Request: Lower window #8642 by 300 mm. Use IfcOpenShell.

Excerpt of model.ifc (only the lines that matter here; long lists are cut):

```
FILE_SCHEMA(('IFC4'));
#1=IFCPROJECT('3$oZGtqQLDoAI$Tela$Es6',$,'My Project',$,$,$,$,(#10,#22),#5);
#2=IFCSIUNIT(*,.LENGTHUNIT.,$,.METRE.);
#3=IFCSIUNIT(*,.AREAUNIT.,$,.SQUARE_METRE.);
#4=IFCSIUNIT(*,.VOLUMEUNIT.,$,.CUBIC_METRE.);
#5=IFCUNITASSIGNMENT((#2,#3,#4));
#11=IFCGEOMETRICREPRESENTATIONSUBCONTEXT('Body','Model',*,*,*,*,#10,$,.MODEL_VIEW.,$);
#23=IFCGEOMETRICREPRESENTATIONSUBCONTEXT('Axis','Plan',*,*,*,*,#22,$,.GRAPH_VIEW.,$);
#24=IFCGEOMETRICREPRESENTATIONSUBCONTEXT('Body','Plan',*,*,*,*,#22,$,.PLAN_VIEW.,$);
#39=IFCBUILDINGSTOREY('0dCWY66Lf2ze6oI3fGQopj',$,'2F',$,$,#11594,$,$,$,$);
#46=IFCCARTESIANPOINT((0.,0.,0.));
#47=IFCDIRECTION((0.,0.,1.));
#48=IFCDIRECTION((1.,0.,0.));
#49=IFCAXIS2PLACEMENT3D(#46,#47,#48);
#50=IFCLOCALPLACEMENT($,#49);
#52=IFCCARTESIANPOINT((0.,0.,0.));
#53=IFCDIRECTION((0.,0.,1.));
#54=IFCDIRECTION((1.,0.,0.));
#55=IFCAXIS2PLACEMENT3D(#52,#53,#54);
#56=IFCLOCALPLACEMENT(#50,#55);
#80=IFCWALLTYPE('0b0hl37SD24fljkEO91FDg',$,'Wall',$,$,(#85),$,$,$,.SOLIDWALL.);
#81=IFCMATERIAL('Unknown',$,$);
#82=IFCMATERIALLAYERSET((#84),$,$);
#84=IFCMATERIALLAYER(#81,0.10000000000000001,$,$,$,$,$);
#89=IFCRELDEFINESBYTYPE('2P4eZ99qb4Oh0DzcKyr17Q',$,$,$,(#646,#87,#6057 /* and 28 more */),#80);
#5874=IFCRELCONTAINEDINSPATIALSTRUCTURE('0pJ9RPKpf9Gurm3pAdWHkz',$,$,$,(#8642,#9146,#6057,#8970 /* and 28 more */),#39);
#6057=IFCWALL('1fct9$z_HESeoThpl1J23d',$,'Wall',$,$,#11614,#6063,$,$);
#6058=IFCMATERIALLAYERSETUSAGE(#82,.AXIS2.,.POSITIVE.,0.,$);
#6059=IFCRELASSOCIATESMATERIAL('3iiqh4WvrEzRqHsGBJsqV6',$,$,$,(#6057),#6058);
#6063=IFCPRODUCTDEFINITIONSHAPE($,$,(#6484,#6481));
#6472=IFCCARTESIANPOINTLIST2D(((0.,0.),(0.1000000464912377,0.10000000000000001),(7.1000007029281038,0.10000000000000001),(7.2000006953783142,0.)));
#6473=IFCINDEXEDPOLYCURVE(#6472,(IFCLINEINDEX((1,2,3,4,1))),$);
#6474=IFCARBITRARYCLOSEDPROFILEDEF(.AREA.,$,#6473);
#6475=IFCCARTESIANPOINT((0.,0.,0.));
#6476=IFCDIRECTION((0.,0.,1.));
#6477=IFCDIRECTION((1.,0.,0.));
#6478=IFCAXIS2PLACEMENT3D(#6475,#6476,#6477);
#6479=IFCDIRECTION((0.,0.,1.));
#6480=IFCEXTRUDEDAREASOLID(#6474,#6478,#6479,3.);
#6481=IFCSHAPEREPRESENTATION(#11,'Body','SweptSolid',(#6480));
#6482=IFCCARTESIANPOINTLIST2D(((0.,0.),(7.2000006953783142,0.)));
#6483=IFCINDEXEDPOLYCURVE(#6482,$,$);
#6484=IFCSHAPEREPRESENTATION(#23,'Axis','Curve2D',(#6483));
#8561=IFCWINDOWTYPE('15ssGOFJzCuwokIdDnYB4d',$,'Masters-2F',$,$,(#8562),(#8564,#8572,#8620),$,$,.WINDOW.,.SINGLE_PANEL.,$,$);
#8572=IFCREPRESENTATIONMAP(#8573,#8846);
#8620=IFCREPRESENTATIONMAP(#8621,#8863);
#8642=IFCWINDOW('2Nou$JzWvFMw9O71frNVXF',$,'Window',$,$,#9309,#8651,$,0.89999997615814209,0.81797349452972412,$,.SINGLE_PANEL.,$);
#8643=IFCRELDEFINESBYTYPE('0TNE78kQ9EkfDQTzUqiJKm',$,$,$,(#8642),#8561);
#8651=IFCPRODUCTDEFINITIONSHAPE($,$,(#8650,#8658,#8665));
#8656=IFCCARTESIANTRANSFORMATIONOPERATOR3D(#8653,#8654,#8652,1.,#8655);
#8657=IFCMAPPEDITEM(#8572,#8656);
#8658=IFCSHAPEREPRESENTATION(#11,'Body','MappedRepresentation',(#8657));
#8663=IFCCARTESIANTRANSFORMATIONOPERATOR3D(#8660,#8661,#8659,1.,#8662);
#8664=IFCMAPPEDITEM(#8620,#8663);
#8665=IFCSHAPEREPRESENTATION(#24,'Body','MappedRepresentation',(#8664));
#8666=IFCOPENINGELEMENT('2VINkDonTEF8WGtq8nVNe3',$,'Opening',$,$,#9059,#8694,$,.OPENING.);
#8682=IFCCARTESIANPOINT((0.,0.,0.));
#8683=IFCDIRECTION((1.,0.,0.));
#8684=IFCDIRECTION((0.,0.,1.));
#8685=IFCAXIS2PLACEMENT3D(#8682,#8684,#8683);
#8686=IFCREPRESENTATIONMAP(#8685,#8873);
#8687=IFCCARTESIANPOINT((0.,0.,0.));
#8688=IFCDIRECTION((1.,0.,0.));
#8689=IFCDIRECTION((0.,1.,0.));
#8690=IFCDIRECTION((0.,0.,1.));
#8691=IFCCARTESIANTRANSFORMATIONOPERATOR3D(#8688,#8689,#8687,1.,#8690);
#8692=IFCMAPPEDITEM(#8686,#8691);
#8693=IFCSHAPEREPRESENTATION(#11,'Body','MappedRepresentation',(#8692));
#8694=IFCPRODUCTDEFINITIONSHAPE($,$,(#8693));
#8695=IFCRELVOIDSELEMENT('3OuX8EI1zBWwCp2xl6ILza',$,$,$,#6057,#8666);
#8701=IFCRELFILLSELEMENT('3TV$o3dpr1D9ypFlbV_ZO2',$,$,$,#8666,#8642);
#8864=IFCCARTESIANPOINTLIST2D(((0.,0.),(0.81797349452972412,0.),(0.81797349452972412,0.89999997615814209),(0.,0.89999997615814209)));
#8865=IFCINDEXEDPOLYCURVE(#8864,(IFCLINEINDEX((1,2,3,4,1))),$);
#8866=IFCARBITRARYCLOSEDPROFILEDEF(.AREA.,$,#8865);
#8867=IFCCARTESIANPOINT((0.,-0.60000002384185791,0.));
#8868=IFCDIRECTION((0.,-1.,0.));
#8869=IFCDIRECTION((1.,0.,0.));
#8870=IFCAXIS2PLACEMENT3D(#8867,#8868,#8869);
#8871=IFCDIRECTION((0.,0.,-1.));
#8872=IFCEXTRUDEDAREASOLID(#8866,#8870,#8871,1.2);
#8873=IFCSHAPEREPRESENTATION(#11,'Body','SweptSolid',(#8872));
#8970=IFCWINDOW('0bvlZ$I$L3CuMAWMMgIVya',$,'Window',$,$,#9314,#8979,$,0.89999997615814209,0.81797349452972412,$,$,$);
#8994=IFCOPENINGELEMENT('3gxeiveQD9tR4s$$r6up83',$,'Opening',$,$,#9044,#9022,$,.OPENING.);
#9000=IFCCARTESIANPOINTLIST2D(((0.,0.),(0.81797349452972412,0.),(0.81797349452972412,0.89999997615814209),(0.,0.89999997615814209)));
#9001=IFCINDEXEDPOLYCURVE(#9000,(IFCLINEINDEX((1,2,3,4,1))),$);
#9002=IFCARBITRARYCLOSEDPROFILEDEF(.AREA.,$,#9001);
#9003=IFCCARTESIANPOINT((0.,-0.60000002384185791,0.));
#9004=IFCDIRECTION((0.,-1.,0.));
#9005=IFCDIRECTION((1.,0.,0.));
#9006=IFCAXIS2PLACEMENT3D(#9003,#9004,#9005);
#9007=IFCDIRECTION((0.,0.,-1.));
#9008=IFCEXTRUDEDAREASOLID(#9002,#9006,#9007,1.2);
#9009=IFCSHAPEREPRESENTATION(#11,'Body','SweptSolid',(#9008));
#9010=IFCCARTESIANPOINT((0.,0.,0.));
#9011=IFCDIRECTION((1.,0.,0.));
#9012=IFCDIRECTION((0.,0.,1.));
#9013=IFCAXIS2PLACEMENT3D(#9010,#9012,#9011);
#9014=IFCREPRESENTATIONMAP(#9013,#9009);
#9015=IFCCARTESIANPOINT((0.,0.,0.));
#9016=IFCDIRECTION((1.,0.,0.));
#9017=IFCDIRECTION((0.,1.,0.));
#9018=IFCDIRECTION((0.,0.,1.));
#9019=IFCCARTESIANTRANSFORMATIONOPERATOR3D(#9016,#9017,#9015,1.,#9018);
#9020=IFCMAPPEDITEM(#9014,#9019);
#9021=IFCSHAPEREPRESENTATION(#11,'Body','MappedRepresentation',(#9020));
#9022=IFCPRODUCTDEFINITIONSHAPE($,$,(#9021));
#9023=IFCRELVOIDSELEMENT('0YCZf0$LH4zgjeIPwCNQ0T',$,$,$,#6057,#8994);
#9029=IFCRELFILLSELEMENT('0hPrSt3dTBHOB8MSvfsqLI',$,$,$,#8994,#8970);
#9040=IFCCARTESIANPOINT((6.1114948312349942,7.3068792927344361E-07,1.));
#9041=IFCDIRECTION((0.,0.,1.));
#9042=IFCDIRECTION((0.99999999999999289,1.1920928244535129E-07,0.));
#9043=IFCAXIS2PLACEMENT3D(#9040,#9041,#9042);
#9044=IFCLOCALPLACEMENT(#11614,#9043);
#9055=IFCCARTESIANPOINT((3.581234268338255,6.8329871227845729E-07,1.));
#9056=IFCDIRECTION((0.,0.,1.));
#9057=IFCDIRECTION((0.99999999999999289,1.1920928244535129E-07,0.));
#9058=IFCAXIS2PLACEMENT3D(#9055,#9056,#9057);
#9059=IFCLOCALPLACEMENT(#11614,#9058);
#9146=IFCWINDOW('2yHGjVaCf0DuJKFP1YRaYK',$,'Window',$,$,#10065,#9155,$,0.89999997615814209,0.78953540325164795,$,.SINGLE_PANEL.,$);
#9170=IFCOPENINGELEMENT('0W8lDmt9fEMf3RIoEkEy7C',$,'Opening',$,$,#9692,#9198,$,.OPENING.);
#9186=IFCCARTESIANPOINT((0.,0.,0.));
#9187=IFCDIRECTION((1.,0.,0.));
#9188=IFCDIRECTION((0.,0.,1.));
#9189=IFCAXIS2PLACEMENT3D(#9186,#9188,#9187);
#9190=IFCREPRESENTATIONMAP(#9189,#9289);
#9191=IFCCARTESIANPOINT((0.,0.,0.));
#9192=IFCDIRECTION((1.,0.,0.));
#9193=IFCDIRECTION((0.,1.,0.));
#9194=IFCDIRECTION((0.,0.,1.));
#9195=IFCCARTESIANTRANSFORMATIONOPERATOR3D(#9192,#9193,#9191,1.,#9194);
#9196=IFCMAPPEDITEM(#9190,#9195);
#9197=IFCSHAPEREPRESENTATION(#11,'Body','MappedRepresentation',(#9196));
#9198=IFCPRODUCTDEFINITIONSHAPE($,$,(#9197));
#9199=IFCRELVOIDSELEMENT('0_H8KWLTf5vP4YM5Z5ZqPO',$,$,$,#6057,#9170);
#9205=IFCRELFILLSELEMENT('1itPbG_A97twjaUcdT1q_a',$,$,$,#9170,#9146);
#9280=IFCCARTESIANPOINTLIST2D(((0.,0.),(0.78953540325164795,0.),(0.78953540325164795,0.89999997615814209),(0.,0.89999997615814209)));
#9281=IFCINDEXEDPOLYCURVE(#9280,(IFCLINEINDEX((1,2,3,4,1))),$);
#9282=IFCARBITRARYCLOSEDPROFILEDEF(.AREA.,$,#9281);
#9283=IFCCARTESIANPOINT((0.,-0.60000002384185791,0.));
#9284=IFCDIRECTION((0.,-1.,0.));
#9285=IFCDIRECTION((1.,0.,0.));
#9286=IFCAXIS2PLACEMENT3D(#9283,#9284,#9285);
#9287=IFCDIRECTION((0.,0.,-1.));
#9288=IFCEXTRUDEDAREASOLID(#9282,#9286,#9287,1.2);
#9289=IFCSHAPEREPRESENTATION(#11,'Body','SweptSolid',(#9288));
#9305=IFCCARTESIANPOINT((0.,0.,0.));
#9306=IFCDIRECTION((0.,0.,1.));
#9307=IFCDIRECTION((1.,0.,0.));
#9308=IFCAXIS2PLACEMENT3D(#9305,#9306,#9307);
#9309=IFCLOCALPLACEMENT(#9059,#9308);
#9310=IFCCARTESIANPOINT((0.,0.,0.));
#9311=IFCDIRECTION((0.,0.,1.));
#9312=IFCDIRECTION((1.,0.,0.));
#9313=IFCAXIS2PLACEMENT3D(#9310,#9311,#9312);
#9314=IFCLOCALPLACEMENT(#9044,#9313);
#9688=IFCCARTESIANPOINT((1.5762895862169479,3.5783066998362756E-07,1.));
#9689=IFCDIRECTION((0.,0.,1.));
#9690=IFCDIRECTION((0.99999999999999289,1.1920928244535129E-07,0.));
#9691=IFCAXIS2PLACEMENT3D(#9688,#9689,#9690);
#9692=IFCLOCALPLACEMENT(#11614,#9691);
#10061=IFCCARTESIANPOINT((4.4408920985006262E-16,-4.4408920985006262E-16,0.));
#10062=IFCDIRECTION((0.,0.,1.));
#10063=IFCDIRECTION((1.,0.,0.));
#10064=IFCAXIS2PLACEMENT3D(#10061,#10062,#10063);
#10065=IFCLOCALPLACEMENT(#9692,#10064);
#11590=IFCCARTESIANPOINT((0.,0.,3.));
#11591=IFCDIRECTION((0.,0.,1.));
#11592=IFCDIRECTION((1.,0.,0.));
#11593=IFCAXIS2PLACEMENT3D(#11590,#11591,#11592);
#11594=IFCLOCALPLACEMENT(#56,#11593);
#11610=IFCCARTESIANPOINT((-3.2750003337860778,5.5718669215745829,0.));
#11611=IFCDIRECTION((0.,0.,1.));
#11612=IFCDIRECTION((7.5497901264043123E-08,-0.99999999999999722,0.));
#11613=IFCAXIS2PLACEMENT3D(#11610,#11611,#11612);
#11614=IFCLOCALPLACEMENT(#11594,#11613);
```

```python
import numpy as np
import ifcopenshell
import ifcopenshell.api.geometry
import ifcopenshell.util.placement
import ifcopenshell.util.unit

model = ifcopenshell.open("model.ifc")
unit_scale = ifcopenshell.util.unit.calculate_unit_scale(model)

window = model.by_id(8642)
opening = window.FillsVoids[0].RelatingOpeningElement
dz = -0.3 / unit_scale

shift = np.array([0.0, 0.0, dz])
# The window is placed relative to its opening, so it follows when the opening moves.
matrix = ifcopenshell.util.placement.get_local_placement(opening.ObjectPlacement)
matrix[:3, 3] += shift
ifcopenshell.api.geometry.edit_object_placement(
    model, product=opening, matrix=matrix, is_si=False, should_transform_children=True
)

print(f"moved by {dz * unit_scale:+.3f} m")

model.write("model_v2.ifc")
```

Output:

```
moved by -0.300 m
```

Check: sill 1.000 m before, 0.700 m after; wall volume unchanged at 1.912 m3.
